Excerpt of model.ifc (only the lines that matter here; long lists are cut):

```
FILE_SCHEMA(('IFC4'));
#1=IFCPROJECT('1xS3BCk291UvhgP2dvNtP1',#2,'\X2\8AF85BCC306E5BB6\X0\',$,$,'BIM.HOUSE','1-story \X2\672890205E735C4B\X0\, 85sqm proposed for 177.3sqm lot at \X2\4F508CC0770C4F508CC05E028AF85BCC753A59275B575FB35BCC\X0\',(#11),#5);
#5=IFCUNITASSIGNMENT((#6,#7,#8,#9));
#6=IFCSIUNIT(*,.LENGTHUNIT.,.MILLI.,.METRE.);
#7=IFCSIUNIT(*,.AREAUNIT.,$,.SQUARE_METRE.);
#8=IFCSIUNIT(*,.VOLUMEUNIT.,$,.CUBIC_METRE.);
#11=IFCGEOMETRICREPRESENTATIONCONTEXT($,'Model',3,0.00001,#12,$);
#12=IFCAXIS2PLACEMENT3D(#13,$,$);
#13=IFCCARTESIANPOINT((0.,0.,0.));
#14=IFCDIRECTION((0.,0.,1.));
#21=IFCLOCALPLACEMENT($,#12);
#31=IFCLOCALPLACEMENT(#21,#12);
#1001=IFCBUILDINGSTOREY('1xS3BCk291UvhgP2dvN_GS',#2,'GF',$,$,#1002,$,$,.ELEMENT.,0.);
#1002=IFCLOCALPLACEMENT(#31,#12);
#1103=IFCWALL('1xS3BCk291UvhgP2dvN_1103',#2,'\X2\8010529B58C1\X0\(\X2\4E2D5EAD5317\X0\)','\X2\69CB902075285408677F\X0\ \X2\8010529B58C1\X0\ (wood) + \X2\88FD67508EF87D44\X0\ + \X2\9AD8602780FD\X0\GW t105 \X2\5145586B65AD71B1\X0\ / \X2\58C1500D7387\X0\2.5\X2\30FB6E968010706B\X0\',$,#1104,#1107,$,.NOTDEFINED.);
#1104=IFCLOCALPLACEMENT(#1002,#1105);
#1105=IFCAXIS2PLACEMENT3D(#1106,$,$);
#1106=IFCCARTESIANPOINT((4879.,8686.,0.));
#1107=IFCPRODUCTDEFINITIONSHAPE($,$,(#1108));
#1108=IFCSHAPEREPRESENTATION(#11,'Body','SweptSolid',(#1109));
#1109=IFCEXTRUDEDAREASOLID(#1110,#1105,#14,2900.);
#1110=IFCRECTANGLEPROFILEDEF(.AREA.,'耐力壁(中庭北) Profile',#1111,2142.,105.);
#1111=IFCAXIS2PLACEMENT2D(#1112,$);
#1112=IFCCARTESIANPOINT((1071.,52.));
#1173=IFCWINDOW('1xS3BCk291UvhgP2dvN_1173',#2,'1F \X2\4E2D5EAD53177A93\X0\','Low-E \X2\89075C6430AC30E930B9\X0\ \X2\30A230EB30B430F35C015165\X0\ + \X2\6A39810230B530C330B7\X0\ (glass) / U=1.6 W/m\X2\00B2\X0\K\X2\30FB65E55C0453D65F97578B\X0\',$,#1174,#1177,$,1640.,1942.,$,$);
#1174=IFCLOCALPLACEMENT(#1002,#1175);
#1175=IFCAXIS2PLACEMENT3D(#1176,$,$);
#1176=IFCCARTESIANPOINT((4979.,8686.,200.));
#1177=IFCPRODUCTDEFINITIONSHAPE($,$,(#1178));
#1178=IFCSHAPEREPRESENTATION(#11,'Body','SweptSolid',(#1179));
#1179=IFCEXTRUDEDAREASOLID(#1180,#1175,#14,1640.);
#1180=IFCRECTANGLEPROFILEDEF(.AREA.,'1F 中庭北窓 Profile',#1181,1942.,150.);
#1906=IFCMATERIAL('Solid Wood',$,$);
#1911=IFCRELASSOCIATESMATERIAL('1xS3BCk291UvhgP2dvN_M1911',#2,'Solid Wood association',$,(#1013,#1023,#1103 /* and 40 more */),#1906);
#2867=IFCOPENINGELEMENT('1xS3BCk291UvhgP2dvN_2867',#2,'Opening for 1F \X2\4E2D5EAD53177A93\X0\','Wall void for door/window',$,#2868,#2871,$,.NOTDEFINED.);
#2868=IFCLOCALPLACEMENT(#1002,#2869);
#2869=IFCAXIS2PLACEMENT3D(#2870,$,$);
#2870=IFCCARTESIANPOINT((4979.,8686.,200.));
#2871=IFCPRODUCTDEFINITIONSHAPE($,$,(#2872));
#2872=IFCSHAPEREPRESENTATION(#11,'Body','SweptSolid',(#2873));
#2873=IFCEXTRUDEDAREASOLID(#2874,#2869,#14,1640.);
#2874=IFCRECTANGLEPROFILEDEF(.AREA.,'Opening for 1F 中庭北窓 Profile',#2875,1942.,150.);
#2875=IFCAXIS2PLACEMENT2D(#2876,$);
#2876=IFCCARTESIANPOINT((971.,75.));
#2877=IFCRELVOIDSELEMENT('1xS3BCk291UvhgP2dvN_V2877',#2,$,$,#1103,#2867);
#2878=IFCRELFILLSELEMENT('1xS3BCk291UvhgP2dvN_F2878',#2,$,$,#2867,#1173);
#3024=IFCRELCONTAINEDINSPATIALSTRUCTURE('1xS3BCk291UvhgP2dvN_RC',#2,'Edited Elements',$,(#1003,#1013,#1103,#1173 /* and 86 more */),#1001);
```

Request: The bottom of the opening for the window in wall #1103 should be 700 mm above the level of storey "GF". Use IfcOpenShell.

```python
import numpy as np
import ifcopenshell
import ifcopenshell.api.geometry
import ifcopenshell.geom
import ifcopenshell.util.element
import ifcopenshell.util.placement
import ifcopenshell.util.shape
import ifcopenshell.util.unit

model = ifcopenshell.open("model.ifc")
unit_scale = ifcopenshell.util.unit.calculate_unit_scale(model)

window = model.by_guid("1xS3BCk291UvhgP2dvN_1173")
opening = window.FillsVoids[0].RelatingOpeningElement
storey = ifcopenshell.util.element.get_container(window, ifc_class="IfcBuildingStorey")
level = ifcopenshell.util.placement.get_local_placement(storey.ObjectPlacement)[2, 3]

# The opening's origin need not be at the sill, so measure its lowest point.
shape = ifcopenshell.geom.create_shape(ifcopenshell.geom.settings(), opening)
bottom = ifcopenshell.util.shape.get_shape_bottom_elevation(shape, shape.geometry) / unit_scale
dz = level + 0.7 / unit_scale - bottom

shift = np.array([0.0, 0.0, dz])
# The window is not placed relative to its opening, so move both.
for product in (opening, window):
    matrix = ifcopenshell.util.placement.get_local_placement(product.ObjectPlacement)
    matrix[:3, 3] += shift
    ifcopenshell.api.geometry.edit_object_placement(model, product=product, matrix=matrix, is_si=False)

print(f"moved by {dz * unit_scale:+.3f} m")

model.write("model-out.ifc")
```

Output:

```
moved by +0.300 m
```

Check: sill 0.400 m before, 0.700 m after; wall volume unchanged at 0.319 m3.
